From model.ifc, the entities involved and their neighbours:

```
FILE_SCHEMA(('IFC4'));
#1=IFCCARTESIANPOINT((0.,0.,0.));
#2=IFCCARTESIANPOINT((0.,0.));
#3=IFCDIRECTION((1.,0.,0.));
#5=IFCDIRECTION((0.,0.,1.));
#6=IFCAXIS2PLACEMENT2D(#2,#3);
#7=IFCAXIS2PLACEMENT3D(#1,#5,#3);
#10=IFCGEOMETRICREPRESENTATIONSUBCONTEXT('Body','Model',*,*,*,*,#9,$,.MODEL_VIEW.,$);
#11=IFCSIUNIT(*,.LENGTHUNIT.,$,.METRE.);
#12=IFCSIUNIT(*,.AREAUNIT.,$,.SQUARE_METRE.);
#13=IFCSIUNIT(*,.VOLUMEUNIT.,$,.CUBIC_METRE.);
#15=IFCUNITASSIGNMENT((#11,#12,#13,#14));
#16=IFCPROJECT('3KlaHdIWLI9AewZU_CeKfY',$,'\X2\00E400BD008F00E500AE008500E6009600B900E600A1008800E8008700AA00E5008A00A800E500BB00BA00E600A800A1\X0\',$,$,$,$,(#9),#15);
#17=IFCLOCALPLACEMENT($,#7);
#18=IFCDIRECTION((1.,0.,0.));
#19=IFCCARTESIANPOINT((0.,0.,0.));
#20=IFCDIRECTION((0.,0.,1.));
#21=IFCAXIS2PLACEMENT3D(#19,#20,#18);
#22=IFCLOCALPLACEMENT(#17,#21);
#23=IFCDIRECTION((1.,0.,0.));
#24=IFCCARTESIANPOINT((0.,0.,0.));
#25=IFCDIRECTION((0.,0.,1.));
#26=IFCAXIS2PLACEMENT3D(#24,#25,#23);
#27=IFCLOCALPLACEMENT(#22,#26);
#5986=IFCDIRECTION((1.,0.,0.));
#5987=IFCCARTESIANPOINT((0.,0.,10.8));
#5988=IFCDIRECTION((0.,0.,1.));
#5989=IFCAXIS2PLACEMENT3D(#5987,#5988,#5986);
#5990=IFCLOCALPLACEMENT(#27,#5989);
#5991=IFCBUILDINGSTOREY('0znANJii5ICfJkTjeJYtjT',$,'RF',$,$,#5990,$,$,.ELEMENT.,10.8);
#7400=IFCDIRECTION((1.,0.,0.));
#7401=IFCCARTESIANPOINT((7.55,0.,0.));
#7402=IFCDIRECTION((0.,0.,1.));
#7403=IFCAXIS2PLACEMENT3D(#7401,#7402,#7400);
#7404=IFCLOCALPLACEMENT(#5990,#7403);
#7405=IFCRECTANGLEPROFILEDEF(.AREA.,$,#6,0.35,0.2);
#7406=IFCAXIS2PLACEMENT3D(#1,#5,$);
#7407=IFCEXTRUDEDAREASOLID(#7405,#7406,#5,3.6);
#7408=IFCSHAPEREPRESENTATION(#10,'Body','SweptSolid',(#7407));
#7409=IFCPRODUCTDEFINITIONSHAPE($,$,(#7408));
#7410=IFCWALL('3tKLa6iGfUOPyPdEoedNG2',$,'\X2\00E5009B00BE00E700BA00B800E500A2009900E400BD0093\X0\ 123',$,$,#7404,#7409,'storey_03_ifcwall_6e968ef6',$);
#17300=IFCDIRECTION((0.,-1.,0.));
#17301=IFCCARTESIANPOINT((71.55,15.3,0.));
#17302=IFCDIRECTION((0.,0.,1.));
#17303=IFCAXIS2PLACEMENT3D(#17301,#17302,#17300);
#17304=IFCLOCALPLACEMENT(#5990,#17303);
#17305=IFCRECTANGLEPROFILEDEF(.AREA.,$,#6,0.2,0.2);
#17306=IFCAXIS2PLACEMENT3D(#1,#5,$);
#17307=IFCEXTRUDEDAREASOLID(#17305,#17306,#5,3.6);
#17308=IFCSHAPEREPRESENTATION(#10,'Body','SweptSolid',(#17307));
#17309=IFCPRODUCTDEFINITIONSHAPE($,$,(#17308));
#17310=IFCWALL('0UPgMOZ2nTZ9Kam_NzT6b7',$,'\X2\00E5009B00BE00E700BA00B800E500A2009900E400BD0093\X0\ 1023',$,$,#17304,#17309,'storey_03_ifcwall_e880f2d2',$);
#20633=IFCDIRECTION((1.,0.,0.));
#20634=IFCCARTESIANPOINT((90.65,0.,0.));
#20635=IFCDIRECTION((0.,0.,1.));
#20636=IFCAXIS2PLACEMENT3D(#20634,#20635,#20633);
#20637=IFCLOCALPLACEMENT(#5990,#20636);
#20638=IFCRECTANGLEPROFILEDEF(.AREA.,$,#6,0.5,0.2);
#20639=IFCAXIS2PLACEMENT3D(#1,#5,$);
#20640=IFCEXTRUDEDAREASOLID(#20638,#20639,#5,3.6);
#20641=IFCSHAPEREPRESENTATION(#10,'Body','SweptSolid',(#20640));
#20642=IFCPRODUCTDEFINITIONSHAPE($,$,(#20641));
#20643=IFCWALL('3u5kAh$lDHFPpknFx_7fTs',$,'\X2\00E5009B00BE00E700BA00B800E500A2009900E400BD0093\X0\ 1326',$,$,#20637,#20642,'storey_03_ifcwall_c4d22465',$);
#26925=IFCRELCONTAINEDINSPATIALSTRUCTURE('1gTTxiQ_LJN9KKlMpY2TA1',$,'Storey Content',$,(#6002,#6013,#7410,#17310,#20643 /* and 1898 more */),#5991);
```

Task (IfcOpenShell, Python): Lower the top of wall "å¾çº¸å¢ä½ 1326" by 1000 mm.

```python
import ifcopenshell
import ifcopenshell.geom
import ifcopenshell.util.representation
import ifcopenshell.util.shape
import ifcopenshell.util.unit

model = ifcopenshell.open("model.ifc")
unit_scale = ifcopenshell.util.unit.calculate_unit_scale(model)
settings = ifcopenshell.geom.settings()


def volume(element):
    """Net volume in cubic metres, openings subtracted."""
    shape = ifcopenshell.geom.create_shape(settings, element)
    return ifcopenshell.util.shape.get_volume(shape.geometry)


wall = model.by_guid("3u5kAh$lDHFPpknFx_7fTs")
before = volume(wall)

body = ifcopenshell.util.representation.get_representation(wall, "Model", "Body")
solid = body.Items[0]
old_height = solid.Depth
solid.Depth -= 1 / unit_scale
after = volume(wall)

print(f"height {old_height:g} -> {solid.Depth:g}, volume {before:.3f} -> {after:.3f} m3")

model.write("model_v2.ifc")
```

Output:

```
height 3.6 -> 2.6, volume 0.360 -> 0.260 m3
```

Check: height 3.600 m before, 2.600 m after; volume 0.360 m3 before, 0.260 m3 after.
